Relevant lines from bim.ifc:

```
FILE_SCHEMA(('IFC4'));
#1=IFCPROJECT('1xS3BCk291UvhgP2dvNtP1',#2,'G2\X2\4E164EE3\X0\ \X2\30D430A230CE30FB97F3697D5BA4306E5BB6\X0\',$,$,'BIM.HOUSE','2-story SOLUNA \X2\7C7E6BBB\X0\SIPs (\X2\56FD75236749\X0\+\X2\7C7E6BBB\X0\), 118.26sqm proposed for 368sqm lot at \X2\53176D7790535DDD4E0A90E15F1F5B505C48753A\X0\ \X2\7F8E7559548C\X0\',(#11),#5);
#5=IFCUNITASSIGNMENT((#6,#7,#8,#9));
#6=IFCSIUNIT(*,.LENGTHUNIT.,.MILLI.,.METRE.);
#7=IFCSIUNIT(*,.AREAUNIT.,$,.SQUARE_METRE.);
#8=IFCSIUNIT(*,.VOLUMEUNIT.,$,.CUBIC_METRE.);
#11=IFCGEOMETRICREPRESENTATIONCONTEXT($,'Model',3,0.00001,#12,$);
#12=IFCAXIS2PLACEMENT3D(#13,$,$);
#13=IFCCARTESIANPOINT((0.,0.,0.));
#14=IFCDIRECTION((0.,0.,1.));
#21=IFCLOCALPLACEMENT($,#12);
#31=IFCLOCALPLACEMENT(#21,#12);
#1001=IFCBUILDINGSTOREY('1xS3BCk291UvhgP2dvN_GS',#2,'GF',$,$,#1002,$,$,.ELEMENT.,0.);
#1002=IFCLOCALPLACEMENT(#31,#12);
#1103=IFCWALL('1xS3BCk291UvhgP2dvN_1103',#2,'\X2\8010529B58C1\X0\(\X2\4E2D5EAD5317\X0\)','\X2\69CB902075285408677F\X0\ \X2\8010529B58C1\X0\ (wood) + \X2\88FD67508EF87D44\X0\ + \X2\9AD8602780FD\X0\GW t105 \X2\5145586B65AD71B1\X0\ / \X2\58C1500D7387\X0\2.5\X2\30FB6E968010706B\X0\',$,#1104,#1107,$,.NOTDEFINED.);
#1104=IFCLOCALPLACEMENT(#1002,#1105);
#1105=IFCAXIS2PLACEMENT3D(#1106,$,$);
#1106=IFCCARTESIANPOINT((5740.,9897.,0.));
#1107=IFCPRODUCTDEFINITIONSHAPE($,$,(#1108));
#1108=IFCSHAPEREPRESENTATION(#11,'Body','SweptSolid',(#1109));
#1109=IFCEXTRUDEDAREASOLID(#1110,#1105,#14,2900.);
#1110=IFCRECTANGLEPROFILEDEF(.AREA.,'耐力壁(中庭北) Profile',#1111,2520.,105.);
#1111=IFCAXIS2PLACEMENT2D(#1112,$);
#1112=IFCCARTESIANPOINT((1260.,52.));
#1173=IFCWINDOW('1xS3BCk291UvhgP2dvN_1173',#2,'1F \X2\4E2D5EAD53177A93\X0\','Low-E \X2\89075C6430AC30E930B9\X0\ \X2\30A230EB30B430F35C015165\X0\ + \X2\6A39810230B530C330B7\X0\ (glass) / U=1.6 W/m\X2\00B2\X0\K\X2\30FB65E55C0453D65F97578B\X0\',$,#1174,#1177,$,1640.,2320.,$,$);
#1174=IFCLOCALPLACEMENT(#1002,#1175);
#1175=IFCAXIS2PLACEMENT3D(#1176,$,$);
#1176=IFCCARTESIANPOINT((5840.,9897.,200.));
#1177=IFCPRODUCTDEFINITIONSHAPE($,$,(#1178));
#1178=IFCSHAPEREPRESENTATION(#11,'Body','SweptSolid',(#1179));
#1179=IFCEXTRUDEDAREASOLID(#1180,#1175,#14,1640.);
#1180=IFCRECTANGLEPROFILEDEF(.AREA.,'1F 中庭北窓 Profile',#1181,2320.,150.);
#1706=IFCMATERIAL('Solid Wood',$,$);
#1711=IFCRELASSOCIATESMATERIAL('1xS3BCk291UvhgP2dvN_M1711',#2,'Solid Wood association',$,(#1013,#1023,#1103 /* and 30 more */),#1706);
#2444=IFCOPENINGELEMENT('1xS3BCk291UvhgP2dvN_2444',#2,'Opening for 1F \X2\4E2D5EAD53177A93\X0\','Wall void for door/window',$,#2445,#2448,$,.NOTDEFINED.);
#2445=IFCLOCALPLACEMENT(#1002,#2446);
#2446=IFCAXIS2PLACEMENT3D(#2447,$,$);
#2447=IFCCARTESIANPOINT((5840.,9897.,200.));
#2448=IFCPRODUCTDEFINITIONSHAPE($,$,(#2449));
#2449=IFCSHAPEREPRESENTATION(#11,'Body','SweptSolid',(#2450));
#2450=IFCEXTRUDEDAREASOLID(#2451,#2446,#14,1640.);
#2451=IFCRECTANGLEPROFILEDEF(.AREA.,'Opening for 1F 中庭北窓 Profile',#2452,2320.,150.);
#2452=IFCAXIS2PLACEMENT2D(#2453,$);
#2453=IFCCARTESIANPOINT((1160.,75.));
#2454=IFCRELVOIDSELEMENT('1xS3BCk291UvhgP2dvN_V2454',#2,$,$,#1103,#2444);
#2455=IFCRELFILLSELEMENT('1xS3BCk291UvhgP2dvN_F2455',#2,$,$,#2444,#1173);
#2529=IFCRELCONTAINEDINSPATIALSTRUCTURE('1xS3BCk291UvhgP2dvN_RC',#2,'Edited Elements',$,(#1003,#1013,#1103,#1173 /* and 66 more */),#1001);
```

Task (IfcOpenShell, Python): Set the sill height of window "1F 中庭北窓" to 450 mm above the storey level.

```python
import numpy as np
import ifcopenshell
import ifcopenshell.api.geometry
import ifcopenshell.geom
import ifcopenshell.util.element
import ifcopenshell.util.placement
import ifcopenshell.util.shape
import ifcopenshell.util.unit

model = ifcopenshell.open("bim.ifc")
unit_scale = ifcopenshell.util.unit.calculate_unit_scale(model)

window = model.by_guid("1xS3BCk291UvhgP2dvN_1173")
opening = window.FillsVoids[0].RelatingOpeningElement
storey = ifcopenshell.util.element.get_container(window, ifc_class="IfcBuildingStorey")
level = ifcopenshell.util.placement.get_local_placement(storey.ObjectPlacement)[2, 3]

# The opening's origin need not be at the sill, so measure its lowest point.
shape = ifcopenshell.geom.create_shape(ifcopenshell.geom.settings(), opening)
bottom = ifcopenshell.util.shape.get_shape_bottom_elevation(shape, shape.geometry) / unit_scale
dz = level + 450.0 - bottom

shift = np.array([0.0, 0.0, dz])
# The window is not placed relative to its opening, so move both.
for product in (opening, window):
    matrix = ifcopenshell.util.placement.get_local_placement(product.ObjectPlacement)
    matrix[:3, 3] += shift
    ifcopenshell.api.geometry.edit_object_placement(model, product=product, matrix=matrix, is_si=False)

print(f"moved by {dz * unit_scale:+.3f} m")

model.write("bim_edited.ifc")
```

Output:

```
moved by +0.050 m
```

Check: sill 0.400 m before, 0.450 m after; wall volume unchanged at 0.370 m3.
